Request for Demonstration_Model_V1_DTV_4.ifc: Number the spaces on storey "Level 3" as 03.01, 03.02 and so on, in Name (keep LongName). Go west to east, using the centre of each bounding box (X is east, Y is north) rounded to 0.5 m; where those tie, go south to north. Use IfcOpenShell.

First a look at what the model holds.

```python
import ifcopenshell
import ifcopenshell.util.element
import ifcopenshell.util.placement

model = ifcopenshell.open("Demonstration_Model_V1_DTV_4.ifc")
print(model.schema)
storey = next(s for s in model.by_type("IfcBuildingStorey") if s.Name == "Level 3")
spaces = [e for e in ifcopenshell.util.element.get_decomposition(storey) if e.is_a("IfcSpace")]
for e in sorted(spaces, key=lambda e: e.id()):
    origin = ifcopenshell.util.placement.get_local_placement(e.ObjectPlacement)[:3, 3]
    print(e.id(), e.Name, e.LongName, origin.round(2) + 0.0, sep=" | ")
```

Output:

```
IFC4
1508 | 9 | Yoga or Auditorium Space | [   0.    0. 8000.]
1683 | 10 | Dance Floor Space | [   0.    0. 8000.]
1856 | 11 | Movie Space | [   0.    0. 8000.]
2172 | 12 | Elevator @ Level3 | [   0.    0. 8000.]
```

```python
import ifcopenshell
import ifcopenshell.geom
import ifcopenshell.util.element
import ifcopenshell.util.shape

model = ifcopenshell.open("Demonstration_Model_V1_DTV_4.ifc")
settings = ifcopenshell.geom.settings()
settings.set("use-world-coords", True)


def centre(element):
    shape = ifcopenshell.geom.create_shape(settings, element)
    return ifcopenshell.util.shape.get_bbox_centroid(shape.geometry)


storey = next(s for s in model.by_type("IfcBuildingStorey") if s.Name == "Level 3")
spaces = [e for e in ifcopenshell.util.element.get_decomposition(storey) if e.is_a("IfcSpace")]

# Insertion points can sit at a corner or the storey origin, so sort by the geometry (in metres).
centres = {e: centre(e) for e in spaces}
spaces.sort(key=lambda e: (round(centres[e][0] / 0.5), centres[e][1]))

for i, e in enumerate(spaces, start=1):
    number = f"03.{i:02d}"
    e.Name = number
    print(e.id(), number)

model.write("Demonstration_Model_V1_DTV_4-out.ifc")
```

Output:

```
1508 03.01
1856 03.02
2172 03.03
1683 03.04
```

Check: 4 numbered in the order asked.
